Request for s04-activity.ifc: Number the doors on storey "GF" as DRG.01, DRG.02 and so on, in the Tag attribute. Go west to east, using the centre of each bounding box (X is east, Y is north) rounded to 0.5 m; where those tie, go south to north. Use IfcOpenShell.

First a look at what the model holds.

```python
import ifcopenshell
import ifcopenshell.util.element
import ifcopenshell.util.placement

model = ifcopenshell.open("s04-activity.ifc")
print(model.schema)
storey = next(s for s in model.by_type("IfcBuildingStorey") if s.Name == "GF")
doors = [e for e in ifcopenshell.util.element.get_decomposition(storey) if e.is_a("IfcDoor")]
for e in sorted(doors, key=lambda e: e.id()):
    origin = ifcopenshell.util.placement.get_local_placement(e.ObjectPlacement)[:3, 3]
    print(e.id(), e.Tag, e.Name, origin.round(2) + 0.0, sep=" | ")
```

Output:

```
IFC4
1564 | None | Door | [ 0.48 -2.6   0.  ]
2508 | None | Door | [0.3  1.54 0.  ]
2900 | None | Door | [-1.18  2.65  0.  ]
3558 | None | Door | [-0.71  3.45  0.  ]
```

```python
import ifcopenshell
import ifcopenshell.geom
import ifcopenshell.util.element
import ifcopenshell.util.shape

model = ifcopenshell.open("s04-activity.ifc")
settings = ifcopenshell.geom.settings()
settings.set("use-world-coords", True)


def centre(element):
    shape = ifcopenshell.geom.create_shape(settings, element)
    return ifcopenshell.util.shape.get_bbox_centroid(shape.geometry)


storey = next(s for s in model.by_type("IfcBuildingStorey") if s.Name == "GF")
doors = [e for e in ifcopenshell.util.element.get_decomposition(storey) if e.is_a("IfcDoor")]

# Insertion points can sit at a corner or the storey origin, so sort by the geometry (in metres).
centres = {e: centre(e) for e in doors}
doors.sort(key=lambda e: (round(centres[e][0] / 0.5), centres[e][1]))

for i, e in enumerate(doors, start=1):
    number = f"DRG.{i:02d}"
    e.Tag = number
    print(e.id(), number)

model.write("s04-activity_edited.ifc")
```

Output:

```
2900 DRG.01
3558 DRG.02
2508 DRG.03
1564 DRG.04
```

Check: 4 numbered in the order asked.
